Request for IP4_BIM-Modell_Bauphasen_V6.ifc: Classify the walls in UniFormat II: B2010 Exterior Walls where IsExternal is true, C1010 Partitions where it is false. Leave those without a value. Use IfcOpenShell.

First a look at what the model holds.

```python
import ifcopenshell
import ifcopenshell.util.element

model = ifcopenshell.open("IP4_BIM-Modell_Bauphasen_V6.ifc")
print(model.schema)
print("classifications:", [c.Name for c in model.by_type("IfcClassification")])
values = [ifcopenshell.util.element.get_pset(e, "Pset_WallCommon", "IsExternal") for e in model.by_type("IfcWall")]
for value in (True, False, None):
    print("IsExternal", value, values.count(value))
```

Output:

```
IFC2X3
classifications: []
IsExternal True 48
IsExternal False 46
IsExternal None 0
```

```python
import ifcopenshell
import ifcopenshell.api.classification
import ifcopenshell.util.element

model = ifcopenshell.open("IP4_BIM-Modell_Bauphasen_V6.ifc")

# IFC2X3 requires Source and Edition and has no link from the project to the system.
system = model.create_entity("IfcClassification", Source="ASTM", Edition="E1557", Name="UniFormat II")

walls = model.by_type("IfcWall")
external = {e: ifcopenshell.util.element.get_pset(e, "Pset_WallCommon", "IsExternal") for e in walls}
for flag, code, name in ((True, "B2010", "Exterior Walls"), (False, "C1010", "Partitions")):
    products = [e for e in walls if external[e] is flag]
    ifcopenshell.api.classification.add_reference(
        model, products=products, classification=system, identification=code, name=name
    )
    print(code, len(products))

model.write("IP4_BIM-Modell_Bauphasen_V6_rev.ifc")
```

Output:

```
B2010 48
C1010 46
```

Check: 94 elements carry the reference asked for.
